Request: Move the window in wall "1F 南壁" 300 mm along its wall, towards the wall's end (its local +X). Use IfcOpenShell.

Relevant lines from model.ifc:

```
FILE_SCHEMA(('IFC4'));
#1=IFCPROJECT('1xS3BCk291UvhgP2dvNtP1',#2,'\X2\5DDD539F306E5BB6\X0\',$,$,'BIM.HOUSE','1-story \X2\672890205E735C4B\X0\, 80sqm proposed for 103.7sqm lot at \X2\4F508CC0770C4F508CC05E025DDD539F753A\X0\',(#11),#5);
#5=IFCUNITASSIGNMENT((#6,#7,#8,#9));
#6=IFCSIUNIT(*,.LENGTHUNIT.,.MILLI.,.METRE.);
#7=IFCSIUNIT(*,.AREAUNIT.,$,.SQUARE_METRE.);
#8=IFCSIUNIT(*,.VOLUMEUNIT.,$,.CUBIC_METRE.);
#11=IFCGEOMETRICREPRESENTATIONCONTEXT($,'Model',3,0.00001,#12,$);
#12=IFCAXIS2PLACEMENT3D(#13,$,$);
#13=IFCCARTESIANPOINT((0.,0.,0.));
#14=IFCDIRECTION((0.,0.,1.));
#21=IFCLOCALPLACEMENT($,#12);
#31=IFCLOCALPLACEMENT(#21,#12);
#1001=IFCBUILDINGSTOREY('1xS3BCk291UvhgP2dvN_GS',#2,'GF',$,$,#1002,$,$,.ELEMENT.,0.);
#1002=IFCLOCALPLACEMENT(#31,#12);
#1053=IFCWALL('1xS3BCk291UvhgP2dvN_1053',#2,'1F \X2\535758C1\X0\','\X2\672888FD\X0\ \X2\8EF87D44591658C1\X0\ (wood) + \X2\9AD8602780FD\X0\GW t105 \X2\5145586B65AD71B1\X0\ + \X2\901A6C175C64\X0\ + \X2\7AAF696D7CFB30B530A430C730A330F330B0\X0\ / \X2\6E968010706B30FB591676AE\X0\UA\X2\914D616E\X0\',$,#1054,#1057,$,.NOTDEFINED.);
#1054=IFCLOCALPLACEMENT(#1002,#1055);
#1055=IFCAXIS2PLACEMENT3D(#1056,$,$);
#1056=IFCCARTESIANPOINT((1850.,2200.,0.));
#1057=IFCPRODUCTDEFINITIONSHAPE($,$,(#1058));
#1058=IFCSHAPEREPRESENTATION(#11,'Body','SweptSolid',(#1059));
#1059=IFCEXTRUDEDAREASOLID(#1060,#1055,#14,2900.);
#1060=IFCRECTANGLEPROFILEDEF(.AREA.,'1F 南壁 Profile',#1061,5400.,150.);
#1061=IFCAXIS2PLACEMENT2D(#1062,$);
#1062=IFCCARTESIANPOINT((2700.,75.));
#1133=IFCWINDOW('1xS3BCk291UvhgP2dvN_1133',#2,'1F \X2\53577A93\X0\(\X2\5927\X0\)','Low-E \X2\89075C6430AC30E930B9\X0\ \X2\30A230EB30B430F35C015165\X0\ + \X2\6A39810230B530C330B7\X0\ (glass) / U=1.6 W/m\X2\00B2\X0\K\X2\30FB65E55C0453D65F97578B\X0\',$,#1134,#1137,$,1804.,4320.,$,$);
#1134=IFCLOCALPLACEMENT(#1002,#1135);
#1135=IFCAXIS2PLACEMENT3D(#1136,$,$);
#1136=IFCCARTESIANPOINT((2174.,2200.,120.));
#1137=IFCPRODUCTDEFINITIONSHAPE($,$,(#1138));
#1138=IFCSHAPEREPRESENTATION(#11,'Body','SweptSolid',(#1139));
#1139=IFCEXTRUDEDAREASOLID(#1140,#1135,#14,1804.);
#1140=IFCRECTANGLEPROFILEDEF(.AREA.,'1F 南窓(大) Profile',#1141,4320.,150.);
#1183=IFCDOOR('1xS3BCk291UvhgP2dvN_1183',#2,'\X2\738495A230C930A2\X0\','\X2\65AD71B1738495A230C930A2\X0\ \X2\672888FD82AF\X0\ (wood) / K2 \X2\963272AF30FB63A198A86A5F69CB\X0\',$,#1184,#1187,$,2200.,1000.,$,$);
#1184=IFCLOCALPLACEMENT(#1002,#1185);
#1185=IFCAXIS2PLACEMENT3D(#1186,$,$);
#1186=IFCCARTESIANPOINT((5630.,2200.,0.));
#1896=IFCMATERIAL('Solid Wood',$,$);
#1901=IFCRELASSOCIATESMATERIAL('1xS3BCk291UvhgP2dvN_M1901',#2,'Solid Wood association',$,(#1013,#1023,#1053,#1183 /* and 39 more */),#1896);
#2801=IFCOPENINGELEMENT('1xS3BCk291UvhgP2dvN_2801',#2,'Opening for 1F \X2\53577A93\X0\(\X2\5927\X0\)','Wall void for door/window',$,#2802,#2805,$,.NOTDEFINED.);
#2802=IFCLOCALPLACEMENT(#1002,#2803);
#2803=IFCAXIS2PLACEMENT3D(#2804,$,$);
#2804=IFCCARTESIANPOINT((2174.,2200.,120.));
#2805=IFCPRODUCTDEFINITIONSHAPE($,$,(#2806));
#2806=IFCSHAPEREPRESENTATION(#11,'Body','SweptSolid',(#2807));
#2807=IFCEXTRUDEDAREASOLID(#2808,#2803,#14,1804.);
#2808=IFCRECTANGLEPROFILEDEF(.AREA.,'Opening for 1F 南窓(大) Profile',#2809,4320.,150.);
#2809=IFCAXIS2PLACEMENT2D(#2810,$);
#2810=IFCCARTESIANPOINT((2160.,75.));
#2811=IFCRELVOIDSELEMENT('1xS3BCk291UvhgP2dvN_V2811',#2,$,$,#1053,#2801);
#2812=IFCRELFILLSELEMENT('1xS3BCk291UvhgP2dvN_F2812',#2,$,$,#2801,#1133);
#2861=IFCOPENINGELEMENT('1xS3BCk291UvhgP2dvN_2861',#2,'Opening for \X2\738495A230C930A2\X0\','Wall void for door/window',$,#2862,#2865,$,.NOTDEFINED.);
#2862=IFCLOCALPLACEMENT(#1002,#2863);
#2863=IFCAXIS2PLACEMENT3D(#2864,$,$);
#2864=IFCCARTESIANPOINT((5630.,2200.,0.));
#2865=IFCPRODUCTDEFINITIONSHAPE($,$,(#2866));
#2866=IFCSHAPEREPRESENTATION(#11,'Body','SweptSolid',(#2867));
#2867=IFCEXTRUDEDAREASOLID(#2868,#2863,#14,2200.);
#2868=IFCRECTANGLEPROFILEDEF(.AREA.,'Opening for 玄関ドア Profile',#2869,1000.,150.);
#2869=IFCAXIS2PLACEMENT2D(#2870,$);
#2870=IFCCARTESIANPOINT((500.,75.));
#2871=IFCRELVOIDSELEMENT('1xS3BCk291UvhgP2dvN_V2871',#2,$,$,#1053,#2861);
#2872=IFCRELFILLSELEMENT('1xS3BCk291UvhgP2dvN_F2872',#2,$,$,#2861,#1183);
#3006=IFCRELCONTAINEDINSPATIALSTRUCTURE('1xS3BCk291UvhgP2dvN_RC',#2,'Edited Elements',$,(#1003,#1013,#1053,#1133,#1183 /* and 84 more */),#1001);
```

```python
import ifcopenshell
import ifcopenshell.api.geometry
import ifcopenshell.util.placement
import ifcopenshell.util.unit

model = ifcopenshell.open("model.ifc")
unit_scale = ifcopenshell.util.unit.calculate_unit_scale(model)

window = model.by_guid("1xS3BCk291UvhgP2dvN_1133")
opening = window.FillsVoids[0].RelatingOpeningElement
wall = opening.VoidsElements[0].RelatingBuildingElement

wall_matrix = ifcopenshell.util.placement.get_local_placement(wall.ObjectPlacement)
shift = wall_matrix[:3, 0] * 0.3 / unit_scale
before = ifcopenshell.util.placement.get_local_placement(window.ObjectPlacement)[:3, 3].copy()

# The window is not placed relative to its opening, so move both.
for product in (opening, window):
    matrix = ifcopenshell.util.placement.get_local_placement(product.ObjectPlacement)
    matrix[:3, 3] += shift
    ifcopenshell.api.geometry.edit_object_placement(model, product=product, matrix=matrix, is_si=False)

after = ifcopenshell.util.placement.get_local_placement(window.ObjectPlacement)[:3, 3]
print("window moved by", (after - before).round(3) + 0.0)

model.write("model-out.ifc")
```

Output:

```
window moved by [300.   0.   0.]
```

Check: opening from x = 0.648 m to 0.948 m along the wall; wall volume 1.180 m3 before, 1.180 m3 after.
